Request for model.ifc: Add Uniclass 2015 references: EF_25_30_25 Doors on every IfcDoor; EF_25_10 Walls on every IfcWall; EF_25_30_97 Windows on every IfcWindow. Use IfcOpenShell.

First a look at what the model holds.

```python
import ifcopenshell

model = ifcopenshell.open("model.ifc")
print(model.schema)
print("classifications:", [c.Name for c in model.by_type("IfcClassification")])
for ifc_class in ("IfcDoor", "IfcRoof", "IfcStair", "IfcWall", "IfcWindow"):
    print(ifc_class, len(model.by_type(ifc_class)))
```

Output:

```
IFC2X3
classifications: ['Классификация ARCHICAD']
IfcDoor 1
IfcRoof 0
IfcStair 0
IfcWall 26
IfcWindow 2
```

```python
import ifcopenshell
import ifcopenshell.api.classification

model = ifcopenshell.open("model.ifc")

# IFC2X3 requires Source and Edition and has no link from the project to the system.
system = model.create_entity("IfcClassification", Source="NBS", Edition="2015", Name="Uniclass 2015")

codes = {
    "IfcDoor": ("EF_25_30_25", "Doors"),
    "IfcWall": ("EF_25_10", "Walls"),
    "IfcWindow": ("EF_25_30_97", "Windows"),
}
for ifc_class, (code, name) in codes.items():
    products = model.by_type(ifc_class)
    ifcopenshell.api.classification.add_reference(
        model, products=products, classification=system, identification=code, name=name
    )
    print(code, len(products))

model.write("model_rev.ifc")
```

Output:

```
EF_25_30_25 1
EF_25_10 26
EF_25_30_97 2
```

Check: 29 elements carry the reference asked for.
